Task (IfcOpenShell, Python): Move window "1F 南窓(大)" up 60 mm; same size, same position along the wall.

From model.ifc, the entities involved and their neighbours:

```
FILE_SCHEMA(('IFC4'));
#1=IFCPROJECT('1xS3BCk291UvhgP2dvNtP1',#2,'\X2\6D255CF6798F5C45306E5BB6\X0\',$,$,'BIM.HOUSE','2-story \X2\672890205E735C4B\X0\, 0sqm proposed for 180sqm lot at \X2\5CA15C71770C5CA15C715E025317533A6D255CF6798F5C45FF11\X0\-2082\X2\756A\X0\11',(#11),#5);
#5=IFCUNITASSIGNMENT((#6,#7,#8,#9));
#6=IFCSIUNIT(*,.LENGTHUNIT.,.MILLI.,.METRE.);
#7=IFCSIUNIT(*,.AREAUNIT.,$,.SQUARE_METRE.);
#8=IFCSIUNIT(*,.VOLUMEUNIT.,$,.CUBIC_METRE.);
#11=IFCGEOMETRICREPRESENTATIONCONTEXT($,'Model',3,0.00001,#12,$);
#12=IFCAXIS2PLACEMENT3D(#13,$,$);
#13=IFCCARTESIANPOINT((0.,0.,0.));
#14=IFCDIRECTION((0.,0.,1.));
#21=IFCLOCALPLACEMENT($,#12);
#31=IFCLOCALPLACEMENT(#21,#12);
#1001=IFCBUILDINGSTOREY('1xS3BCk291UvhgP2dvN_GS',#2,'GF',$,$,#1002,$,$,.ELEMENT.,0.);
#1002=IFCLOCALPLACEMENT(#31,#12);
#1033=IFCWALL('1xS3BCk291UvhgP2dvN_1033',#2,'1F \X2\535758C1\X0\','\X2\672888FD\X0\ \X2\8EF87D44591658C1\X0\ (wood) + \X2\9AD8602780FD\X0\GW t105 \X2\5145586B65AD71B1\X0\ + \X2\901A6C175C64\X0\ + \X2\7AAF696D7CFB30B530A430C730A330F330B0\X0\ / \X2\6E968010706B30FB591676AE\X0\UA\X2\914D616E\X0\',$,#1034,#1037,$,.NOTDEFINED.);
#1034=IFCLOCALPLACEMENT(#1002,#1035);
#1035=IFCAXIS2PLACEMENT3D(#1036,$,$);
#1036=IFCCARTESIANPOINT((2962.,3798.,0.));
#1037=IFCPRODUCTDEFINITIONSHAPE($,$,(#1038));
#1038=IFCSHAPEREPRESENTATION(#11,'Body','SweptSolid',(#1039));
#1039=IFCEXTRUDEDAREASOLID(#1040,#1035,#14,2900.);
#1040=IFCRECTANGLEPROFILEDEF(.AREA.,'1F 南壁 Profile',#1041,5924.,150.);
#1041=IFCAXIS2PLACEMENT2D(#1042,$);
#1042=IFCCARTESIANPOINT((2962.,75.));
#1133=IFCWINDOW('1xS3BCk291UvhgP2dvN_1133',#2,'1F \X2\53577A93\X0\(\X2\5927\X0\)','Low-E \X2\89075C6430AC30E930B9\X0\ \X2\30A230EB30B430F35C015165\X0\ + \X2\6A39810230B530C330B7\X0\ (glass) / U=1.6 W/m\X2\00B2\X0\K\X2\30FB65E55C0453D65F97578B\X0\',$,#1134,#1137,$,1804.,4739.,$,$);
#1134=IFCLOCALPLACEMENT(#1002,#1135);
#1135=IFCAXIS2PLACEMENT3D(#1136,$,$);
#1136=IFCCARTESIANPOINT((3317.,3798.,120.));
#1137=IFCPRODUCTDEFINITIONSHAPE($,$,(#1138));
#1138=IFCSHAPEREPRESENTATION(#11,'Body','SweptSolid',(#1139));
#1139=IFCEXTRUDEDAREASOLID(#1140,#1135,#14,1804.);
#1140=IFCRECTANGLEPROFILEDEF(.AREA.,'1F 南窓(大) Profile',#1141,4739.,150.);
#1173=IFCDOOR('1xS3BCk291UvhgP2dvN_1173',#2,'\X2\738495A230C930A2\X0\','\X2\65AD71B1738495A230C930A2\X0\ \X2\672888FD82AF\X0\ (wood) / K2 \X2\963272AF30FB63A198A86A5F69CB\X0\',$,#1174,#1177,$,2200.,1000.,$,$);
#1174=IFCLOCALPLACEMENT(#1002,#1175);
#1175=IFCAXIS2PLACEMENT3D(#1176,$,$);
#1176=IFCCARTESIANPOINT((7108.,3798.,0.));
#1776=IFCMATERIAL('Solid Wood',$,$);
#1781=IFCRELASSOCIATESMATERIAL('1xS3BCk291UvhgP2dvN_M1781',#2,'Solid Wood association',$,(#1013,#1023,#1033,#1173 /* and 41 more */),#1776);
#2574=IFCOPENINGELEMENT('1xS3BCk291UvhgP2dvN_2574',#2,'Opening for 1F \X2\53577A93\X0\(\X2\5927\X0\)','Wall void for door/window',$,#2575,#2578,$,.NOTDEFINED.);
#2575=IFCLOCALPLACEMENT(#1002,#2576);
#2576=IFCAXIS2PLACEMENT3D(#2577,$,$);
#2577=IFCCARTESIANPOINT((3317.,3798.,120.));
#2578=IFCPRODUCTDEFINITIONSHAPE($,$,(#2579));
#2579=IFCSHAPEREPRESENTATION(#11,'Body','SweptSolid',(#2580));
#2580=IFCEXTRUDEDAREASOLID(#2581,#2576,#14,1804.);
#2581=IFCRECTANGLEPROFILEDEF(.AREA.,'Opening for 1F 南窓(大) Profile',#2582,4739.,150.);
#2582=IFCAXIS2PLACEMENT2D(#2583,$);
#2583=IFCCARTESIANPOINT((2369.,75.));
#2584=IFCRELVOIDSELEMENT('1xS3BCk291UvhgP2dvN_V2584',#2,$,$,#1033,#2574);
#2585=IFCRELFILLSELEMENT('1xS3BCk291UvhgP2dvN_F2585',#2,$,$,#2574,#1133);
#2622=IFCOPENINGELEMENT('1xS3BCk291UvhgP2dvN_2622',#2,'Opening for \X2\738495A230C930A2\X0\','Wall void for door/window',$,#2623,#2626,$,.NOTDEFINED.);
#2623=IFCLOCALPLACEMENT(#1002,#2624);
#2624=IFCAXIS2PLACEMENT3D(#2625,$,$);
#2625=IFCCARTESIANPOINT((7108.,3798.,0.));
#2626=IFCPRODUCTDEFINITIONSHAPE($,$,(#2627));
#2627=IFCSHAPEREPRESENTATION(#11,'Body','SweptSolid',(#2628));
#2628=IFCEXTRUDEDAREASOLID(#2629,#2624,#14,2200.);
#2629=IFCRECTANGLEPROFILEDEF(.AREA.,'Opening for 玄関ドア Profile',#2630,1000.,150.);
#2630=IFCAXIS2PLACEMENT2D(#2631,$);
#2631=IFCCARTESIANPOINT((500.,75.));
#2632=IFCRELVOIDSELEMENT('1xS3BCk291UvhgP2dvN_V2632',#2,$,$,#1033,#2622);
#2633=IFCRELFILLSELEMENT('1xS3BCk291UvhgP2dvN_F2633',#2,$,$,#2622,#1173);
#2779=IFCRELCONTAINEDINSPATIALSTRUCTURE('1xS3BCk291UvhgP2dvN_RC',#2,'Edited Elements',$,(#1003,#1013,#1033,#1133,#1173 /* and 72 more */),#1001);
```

```python
import numpy as np
import ifcopenshell
import ifcopenshell.api.geometry
import ifcopenshell.util.placement
import ifcopenshell.util.unit

model = ifcopenshell.open("model.ifc")
unit_scale = ifcopenshell.util.unit.calculate_unit_scale(model)

window = model.by_id(1133)
opening = window.FillsVoids[0].RelatingOpeningElement
dz = 0.06 / unit_scale

shift = np.array([0.0, 0.0, dz])
# The window is not placed relative to its opening, so move both.
for product in (opening, window):
    matrix = ifcopenshell.util.placement.get_local_placement(product.ObjectPlacement)
    matrix[:3, 3] += shift
    ifcopenshell.api.geometry.edit_object_placement(model, product=product, matrix=matrix, is_si=False)

print(f"moved by {dz * unit_scale:+.3f} m")

model.write("model_v2.ifc")
```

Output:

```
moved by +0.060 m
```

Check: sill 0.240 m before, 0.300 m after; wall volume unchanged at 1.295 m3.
